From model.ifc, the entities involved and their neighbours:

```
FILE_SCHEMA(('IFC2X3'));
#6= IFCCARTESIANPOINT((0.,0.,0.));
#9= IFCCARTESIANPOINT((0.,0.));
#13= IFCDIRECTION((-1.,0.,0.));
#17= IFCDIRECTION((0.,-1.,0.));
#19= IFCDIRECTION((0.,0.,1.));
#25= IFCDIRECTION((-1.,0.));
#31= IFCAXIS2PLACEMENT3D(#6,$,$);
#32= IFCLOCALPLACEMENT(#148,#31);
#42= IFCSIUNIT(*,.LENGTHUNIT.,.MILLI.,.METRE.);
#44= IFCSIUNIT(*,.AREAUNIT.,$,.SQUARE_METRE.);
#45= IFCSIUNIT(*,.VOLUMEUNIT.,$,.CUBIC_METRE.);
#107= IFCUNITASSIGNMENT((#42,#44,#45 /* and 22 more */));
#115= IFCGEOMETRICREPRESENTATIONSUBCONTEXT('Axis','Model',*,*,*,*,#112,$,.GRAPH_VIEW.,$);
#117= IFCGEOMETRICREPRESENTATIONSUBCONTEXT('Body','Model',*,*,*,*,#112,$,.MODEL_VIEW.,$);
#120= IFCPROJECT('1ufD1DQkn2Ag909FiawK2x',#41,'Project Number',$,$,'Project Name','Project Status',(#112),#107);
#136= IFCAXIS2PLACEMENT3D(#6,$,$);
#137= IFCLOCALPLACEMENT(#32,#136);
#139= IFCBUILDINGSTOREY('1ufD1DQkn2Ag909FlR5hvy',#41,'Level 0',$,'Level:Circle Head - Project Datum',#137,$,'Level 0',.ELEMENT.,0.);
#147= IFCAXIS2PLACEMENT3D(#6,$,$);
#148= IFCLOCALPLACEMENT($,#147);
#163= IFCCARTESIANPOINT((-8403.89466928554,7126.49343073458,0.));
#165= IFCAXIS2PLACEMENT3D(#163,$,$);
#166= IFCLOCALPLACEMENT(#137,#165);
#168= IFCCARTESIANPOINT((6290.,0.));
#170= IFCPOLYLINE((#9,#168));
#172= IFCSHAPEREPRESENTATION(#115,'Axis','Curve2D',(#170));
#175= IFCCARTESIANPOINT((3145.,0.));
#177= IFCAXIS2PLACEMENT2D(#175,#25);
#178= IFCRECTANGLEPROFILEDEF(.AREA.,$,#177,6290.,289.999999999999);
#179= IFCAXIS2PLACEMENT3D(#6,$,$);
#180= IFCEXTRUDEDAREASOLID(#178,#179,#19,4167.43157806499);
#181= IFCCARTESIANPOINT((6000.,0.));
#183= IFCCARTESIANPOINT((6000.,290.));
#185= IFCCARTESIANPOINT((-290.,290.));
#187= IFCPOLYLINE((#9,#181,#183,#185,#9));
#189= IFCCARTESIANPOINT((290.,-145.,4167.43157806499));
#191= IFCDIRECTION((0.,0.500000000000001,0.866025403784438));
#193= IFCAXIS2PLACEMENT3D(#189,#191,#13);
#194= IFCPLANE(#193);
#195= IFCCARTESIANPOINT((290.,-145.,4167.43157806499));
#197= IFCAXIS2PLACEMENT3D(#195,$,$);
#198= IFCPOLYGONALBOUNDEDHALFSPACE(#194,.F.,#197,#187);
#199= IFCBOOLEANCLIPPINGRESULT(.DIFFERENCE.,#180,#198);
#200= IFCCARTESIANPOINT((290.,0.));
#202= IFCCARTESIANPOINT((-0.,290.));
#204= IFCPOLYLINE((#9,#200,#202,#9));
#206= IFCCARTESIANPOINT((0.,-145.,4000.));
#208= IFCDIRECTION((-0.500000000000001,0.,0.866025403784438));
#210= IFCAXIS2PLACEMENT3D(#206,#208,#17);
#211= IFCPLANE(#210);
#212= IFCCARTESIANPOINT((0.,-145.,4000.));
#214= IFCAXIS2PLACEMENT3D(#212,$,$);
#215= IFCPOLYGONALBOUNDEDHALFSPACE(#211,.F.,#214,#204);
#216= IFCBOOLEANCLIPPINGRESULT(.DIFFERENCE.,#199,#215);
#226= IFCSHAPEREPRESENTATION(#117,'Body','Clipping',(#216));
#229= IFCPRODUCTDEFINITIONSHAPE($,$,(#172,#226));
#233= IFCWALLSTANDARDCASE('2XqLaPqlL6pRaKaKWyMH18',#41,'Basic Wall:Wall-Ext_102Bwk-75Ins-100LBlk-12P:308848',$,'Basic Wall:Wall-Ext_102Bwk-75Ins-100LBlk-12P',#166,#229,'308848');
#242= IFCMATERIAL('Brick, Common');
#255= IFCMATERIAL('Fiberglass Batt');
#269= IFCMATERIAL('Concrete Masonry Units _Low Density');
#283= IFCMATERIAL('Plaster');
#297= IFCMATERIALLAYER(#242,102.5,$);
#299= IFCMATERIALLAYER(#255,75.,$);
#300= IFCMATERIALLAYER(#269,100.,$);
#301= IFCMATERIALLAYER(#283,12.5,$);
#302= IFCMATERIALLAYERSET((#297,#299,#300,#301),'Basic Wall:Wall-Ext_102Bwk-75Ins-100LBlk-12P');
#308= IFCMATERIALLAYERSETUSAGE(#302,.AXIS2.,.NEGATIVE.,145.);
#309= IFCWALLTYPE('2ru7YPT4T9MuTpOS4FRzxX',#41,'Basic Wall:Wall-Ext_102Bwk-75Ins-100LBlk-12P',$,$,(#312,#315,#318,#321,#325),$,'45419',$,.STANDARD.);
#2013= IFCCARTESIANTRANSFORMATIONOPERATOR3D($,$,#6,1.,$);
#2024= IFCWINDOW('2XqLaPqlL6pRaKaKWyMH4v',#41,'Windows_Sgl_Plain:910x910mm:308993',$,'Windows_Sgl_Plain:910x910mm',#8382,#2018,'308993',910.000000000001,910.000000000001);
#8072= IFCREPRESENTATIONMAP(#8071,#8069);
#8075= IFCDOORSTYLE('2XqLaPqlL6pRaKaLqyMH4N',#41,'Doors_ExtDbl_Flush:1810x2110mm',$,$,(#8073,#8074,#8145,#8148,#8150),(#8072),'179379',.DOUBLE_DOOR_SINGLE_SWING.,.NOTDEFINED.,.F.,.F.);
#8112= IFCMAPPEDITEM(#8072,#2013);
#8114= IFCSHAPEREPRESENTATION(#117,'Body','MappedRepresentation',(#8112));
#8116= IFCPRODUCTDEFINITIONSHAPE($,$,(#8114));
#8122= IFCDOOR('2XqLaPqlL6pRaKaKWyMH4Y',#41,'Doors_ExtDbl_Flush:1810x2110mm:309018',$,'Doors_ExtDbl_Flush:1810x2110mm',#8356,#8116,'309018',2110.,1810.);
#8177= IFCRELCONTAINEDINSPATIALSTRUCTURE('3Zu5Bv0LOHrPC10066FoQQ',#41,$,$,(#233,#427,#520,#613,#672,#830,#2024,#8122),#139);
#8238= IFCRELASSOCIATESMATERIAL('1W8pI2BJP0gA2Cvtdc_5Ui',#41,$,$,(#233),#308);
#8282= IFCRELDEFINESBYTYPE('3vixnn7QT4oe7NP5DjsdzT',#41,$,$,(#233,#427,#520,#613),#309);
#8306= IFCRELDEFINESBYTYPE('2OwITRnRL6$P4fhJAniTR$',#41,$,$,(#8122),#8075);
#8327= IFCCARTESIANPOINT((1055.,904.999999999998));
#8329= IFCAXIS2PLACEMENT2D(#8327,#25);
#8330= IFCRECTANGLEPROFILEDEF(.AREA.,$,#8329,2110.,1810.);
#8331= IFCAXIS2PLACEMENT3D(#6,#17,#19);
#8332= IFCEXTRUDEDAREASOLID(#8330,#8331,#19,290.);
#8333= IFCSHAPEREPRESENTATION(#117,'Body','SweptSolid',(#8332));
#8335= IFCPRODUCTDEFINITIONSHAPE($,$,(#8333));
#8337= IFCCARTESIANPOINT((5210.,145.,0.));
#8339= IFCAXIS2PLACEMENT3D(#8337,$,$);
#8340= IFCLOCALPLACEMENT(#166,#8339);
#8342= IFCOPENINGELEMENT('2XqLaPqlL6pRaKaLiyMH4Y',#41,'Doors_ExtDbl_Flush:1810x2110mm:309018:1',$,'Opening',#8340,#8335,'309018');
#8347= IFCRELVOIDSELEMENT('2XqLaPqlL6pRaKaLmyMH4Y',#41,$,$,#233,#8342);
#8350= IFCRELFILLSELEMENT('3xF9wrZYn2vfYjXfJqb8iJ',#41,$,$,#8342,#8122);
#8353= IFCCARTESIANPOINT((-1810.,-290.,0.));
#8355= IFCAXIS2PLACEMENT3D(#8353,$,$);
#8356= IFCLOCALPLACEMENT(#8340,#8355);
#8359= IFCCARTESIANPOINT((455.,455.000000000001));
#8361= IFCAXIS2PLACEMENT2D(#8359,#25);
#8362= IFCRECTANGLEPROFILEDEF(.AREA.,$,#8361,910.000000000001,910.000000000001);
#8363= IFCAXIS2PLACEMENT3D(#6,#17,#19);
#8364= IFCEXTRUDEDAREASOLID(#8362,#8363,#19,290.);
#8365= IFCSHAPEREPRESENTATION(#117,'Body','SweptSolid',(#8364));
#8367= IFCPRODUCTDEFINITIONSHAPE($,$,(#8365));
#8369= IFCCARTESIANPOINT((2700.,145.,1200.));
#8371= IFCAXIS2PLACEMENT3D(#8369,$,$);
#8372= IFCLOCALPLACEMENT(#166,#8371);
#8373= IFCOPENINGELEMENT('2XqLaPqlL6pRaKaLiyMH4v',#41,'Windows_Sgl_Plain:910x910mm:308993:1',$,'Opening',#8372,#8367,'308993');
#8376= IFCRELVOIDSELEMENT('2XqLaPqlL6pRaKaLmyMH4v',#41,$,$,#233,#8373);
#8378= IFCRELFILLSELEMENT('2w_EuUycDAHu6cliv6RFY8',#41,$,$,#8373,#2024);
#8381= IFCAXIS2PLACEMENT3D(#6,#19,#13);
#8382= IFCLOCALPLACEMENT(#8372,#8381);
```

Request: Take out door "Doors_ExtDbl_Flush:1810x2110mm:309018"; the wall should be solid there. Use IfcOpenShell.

```python
import ifcopenshell
import ifcopenshell.api.feature
import ifcopenshell.api.root
import ifcopenshell.geom
import ifcopenshell.util.shape

model = ifcopenshell.open("model.ifc")
settings = ifcopenshell.geom.settings()


def volume(element):
    """Net volume in cubic metres, openings subtracted."""
    shape = ifcopenshell.geom.create_shape(settings, element)
    return ifcopenshell.util.shape.get_volume(shape.geometry)


door = model.by_guid("2XqLaPqlL6pRaKaKWyMH4Y")
opening = door.FillsVoids[0].RelatingOpeningElement
wall = opening.VoidsElements[0].RelatingBuildingElement
before = volume(wall)

ifcopenshell.api.root.remove_product(model, product=door)
ifcopenshell.api.feature.remove_feature(model, feature=opening)

after = volume(wall)

print(f"wall volume {before:.3f} -> {after:.3f} m3")

model.write("model_updated.ifc")
```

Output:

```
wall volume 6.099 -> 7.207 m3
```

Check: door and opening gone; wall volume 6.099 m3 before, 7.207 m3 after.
